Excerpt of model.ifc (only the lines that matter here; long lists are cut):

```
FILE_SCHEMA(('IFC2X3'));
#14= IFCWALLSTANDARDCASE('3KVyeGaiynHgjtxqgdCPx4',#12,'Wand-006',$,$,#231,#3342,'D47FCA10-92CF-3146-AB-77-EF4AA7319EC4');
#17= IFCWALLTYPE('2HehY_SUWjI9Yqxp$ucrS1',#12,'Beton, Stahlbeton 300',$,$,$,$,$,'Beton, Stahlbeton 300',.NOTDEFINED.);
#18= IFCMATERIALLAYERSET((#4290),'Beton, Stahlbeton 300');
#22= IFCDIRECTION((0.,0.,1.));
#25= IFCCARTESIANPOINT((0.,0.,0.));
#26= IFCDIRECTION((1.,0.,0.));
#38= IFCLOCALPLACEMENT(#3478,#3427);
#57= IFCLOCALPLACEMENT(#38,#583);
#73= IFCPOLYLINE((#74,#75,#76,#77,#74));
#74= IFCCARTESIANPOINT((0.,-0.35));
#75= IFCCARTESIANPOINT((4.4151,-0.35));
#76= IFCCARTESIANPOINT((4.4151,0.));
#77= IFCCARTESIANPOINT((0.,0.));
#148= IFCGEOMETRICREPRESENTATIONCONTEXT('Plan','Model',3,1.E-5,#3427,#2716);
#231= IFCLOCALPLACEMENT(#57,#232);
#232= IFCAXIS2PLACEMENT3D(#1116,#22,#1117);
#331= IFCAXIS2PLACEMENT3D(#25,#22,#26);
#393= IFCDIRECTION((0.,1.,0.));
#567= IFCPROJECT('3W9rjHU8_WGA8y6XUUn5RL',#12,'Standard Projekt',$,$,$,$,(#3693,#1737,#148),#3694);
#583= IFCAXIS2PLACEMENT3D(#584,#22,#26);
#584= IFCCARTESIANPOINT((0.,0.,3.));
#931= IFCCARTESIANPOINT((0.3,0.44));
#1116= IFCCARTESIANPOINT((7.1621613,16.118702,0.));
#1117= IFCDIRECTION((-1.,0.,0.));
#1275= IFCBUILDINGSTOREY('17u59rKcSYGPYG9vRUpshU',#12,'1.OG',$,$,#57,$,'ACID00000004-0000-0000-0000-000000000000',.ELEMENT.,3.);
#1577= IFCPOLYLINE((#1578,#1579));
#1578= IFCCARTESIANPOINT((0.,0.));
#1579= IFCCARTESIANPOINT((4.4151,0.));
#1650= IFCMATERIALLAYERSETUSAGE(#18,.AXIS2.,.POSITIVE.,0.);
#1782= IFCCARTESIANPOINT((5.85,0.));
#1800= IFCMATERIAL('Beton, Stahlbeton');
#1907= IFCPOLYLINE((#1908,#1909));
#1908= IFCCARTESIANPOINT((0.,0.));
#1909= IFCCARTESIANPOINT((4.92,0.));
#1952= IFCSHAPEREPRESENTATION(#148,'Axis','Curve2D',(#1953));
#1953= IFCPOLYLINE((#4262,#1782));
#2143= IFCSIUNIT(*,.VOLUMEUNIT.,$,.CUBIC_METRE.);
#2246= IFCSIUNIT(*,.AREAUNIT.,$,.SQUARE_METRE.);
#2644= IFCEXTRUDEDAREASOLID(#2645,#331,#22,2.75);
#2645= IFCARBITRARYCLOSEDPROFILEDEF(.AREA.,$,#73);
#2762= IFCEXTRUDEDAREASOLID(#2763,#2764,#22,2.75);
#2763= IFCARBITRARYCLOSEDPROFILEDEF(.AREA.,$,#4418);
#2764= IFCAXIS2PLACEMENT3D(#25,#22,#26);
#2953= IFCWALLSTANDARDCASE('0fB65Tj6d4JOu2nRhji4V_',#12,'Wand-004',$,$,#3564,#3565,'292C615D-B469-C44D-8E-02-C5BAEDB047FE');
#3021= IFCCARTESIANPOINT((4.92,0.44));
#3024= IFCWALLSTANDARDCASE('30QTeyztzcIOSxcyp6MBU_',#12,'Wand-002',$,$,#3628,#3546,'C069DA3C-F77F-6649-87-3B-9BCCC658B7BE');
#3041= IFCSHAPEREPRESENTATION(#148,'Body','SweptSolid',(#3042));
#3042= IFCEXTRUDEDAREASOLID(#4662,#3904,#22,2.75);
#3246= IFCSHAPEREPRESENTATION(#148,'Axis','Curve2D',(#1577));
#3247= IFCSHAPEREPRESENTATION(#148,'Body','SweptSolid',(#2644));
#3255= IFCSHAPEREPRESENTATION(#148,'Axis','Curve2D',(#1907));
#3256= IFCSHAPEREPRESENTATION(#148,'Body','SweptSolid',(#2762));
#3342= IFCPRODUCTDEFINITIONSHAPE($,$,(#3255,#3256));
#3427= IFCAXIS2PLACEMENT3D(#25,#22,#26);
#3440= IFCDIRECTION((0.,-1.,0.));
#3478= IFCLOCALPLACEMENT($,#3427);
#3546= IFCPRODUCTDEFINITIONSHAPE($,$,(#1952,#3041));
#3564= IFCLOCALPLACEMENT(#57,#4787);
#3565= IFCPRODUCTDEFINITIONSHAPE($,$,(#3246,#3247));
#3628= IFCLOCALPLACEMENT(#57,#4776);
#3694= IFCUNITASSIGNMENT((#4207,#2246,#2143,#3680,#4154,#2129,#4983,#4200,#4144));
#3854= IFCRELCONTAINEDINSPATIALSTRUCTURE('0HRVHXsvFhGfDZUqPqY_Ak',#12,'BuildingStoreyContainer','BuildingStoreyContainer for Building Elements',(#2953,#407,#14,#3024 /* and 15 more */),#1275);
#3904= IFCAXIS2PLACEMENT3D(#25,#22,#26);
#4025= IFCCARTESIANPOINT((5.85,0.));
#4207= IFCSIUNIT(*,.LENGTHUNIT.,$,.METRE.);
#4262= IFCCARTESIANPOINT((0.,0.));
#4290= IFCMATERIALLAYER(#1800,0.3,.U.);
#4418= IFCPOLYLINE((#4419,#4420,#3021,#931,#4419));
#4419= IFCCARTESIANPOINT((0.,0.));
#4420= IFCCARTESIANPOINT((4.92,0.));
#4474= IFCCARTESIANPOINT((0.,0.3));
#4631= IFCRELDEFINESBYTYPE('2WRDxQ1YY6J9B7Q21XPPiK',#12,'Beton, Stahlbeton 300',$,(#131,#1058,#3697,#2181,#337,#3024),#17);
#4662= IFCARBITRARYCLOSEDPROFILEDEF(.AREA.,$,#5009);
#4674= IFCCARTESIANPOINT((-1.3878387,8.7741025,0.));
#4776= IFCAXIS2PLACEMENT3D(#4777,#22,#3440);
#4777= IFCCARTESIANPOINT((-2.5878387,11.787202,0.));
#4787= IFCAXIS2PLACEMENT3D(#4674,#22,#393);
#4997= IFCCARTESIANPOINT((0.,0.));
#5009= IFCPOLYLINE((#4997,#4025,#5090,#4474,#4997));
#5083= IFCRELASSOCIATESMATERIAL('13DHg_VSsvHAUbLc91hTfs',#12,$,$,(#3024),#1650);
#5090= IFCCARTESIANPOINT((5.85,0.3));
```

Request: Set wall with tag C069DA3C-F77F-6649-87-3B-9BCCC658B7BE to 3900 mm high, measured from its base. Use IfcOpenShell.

```python
import ifcopenshell
import ifcopenshell.geom
import ifcopenshell.util.shape
import ifcopenshell.util.unit

model = ifcopenshell.open("model.ifc")
unit_scale = ifcopenshell.util.unit.calculate_unit_scale(model)
settings = ifcopenshell.geom.settings()


def volume(element):
    """Net volume in cubic metres, openings subtracted."""
    shape = ifcopenshell.geom.create_shape(settings, element)
    return ifcopenshell.util.shape.get_volume(shape.geometry)


wall = model.by_guid("30QTeyztzcIOSxcyp6MBU_")
before = volume(wall)

body = next(r for r in wall.Representation.Representations if r.RepresentationIdentifier == "Body")
solid = body.Items[0]
old_height = solid.Depth
solid.Depth = 3.9 / unit_scale
after = volume(wall)

print(f"height {old_height:g} -> {solid.Depth:g}, volume {before:.3f} -> {after:.3f} m3")

model.write("model_edited.ifc")
```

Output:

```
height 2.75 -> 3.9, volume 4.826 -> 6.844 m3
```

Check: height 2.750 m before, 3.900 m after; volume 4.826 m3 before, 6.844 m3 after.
